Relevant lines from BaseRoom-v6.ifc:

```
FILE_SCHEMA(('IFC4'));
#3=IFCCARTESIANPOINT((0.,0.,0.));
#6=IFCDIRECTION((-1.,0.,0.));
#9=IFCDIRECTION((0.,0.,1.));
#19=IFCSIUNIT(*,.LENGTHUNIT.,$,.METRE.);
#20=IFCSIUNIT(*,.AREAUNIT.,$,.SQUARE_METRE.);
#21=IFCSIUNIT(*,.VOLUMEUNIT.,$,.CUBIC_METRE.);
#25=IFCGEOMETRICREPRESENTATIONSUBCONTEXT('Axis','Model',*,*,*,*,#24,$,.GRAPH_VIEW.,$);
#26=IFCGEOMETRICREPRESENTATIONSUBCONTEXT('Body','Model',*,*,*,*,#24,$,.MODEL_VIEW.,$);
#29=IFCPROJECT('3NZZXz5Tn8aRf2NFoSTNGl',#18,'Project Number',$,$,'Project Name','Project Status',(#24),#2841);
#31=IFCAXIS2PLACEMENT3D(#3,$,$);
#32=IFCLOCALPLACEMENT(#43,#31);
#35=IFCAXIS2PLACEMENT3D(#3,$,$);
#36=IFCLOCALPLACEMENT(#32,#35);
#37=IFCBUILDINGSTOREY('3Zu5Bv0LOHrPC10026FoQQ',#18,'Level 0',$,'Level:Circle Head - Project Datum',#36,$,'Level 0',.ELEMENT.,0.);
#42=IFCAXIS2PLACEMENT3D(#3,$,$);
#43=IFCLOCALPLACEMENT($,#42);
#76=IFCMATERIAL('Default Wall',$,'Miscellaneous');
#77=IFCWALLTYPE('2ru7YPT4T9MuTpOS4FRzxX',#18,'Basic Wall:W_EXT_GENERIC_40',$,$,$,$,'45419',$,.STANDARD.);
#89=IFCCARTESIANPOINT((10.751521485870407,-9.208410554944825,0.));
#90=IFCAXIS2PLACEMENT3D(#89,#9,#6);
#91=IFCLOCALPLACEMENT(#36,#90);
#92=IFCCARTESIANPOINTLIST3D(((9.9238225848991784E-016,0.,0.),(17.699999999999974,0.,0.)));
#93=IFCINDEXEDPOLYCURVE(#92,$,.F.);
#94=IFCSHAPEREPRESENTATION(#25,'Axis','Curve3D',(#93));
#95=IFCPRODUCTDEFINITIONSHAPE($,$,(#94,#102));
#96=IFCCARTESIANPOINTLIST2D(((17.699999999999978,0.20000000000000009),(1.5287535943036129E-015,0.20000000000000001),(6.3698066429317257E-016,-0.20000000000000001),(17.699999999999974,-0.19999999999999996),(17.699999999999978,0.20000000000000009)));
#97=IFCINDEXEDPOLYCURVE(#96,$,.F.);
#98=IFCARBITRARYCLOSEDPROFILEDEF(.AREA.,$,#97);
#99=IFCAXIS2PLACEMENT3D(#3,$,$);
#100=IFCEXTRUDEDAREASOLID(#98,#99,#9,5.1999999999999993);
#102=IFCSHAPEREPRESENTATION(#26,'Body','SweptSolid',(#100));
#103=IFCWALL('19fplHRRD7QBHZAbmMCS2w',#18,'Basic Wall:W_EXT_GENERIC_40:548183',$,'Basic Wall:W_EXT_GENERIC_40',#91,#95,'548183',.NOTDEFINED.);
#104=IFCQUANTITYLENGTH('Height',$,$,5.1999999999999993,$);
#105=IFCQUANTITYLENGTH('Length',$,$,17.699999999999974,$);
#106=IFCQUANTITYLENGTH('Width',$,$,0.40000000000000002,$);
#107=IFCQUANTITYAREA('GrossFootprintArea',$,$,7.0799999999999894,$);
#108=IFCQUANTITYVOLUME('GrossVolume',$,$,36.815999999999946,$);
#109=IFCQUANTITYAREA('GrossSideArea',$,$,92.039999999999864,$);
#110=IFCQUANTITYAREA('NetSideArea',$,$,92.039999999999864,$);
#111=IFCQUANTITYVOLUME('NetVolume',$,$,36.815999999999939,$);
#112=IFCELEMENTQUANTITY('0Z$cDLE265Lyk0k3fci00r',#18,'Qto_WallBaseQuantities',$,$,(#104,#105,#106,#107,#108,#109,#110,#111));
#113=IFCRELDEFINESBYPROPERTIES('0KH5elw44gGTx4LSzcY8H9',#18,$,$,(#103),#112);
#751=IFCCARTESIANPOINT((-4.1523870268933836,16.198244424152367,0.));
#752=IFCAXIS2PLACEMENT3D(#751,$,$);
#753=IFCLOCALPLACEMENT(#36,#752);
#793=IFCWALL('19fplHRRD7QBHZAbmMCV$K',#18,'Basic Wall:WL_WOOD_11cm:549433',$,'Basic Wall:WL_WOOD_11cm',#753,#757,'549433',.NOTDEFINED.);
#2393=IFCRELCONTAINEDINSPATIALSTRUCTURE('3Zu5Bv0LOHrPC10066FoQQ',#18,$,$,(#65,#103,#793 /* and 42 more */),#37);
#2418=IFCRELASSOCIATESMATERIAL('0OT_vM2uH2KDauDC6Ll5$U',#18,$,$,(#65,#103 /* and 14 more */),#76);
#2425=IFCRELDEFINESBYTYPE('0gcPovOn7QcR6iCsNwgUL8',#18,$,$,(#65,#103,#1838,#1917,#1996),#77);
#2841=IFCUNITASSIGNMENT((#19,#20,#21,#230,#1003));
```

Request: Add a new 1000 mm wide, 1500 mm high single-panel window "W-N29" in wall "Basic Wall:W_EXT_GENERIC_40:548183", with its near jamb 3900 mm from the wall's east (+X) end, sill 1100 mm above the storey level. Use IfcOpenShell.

```python
import numpy as np
import ifcopenshell
import ifcopenshell.api.feature
import ifcopenshell.api.geometry
import ifcopenshell.api.pset
import ifcopenshell.api.root
import ifcopenshell.api.spatial
import ifcopenshell.geom
import ifcopenshell.util.element
import ifcopenshell.util.placement
import ifcopenshell.util.representation
import ifcopenshell.util.shape
import ifcopenshell.util.unit

model = ifcopenshell.open("BaseRoom-v6.ifc")
unit_scale = ifcopenshell.util.unit.calculate_unit_scale(model)
area_scale = ifcopenshell.util.unit.calculate_unit_scale(model, "AREAUNIT")
volume_scale = ifcopenshell.util.unit.calculate_unit_scale(model, "VOLUMEUNIT")
settings = ifcopenshell.geom.settings()


def volume(element):
    """Net volume in cubic metres, openings subtracted."""
    shape = ifcopenshell.geom.create_shape(settings, element)
    return ifcopenshell.util.shape.get_volume(shape.geometry)


wall = model.by_guid("19fplHRRD7QBHZAbmMCS2w")
storey = ifcopenshell.util.element.get_container(wall, ifc_class="IfcBuildingStorey")
context = ifcopenshell.util.representation.get_context(model, "Model", "Body", "MODEL_VIEW")
before = volume(wall)

width, height, from_end, sill = 1, 1.5, 3.9, 1.1  # metres

# The wall runs along its own X axis, and the end named is its -X end.
wall_shape = ifcopenshell.geom.create_shape(settings, wall)
x, y, z = ifcopenshell.util.shape.get_vertices(wall_shape.geometry).T
start = x.min() + from_end
face, thickness = float(y.min()), float(y.max() - y.min())
wall_matrix = ifcopenshell.util.placement.get_local_placement(wall.ObjectPlacement)
level = ifcopenshell.util.placement.get_local_placement(storey.ObjectPlacement)[2, 3]


def in_wall(x, y):
    """Placement at x, y metres in the wall's axes, at sill height."""
    matrix = wall_matrix.copy()
    matrix[:, 3] = wall_matrix @ np.array([x / unit_scale, y / unit_scale, 0.0, 1.0])
    matrix[2, 3] = level + sill / unit_scale
    return matrix


# Opening: a box that overshoots both wall faces by 50 mm.
opening = ifcopenshell.api.root.create_entity(model, ifc_class="IfcOpeningElement", predefined_type="OPENING")
box = ifcopenshell.api.geometry.add_wall_representation(
    model, context=context, length=width, height=height, thickness=thickness + 0.1
)
ifcopenshell.api.geometry.assign_representation(model, product=opening, representation=box)
ifcopenshell.api.geometry.edit_object_placement(model, product=opening, matrix=in_wall(start, face - 0.05), is_si=False)
ifcopenshell.api.feature.add_feature(model, feature=opening, element=wall)

window = ifcopenshell.api.root.create_entity(model, ifc_class="IfcWindow", name="W-N29", predefined_type="WINDOW")
window.OverallWidth, window.OverallHeight = width / unit_scale, height / unit_scale
window.PartitioningType = "SINGLE_PANEL"
body = ifcopenshell.api.geometry.add_window_representation(
    model,
    context=context,
    overall_width=window.OverallWidth,
    overall_height=window.OverallHeight,
    partition_type="SINGLE_PANEL",
)
ifcopenshell.api.geometry.assign_representation(model, product=window, representation=body)
ifcopenshell.api.spatial.assign_container(model, products=[window], relating_structure=storey)
ifcopenshell.api.feature.add_filling(model, opening=opening, element=window)

# Centre the window in the wall's thickness.
ifcopenshell.api.geometry.edit_object_placement(model, product=window, matrix=in_wall(start, face), is_si=False)
window_shape = ifcopenshell.geom.create_shape(settings, window)
depth = ifcopenshell.util.shape.get_vertices(window_shape.geometry)[:, 1]
offset = face + thickness / 2 - (depth.min() + depth.max()) / 2
ifcopenshell.api.geometry.edit_object_placement(model, product=window, matrix=in_wall(start, offset), is_si=False)

after = volume(wall)

# Update the wall's stored quantities.
qto = model.by_id(ifcopenshell.util.element.get_pset(wall, "Qto_WallBaseQuantities", should_inherit=False)["id"])
ifcopenshell.api.pset.edit_qto(model, qto=qto, properties={
    "NetSideArea": after / thickness / area_scale,
    "NetVolume": after / volume_scale,
})

print(f"wall volume {before:.3f} -> {after:.3f} m3")

model.write("BaseRoom-v6_edited.ifc")
```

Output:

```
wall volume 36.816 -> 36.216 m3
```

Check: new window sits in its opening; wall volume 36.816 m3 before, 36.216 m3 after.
